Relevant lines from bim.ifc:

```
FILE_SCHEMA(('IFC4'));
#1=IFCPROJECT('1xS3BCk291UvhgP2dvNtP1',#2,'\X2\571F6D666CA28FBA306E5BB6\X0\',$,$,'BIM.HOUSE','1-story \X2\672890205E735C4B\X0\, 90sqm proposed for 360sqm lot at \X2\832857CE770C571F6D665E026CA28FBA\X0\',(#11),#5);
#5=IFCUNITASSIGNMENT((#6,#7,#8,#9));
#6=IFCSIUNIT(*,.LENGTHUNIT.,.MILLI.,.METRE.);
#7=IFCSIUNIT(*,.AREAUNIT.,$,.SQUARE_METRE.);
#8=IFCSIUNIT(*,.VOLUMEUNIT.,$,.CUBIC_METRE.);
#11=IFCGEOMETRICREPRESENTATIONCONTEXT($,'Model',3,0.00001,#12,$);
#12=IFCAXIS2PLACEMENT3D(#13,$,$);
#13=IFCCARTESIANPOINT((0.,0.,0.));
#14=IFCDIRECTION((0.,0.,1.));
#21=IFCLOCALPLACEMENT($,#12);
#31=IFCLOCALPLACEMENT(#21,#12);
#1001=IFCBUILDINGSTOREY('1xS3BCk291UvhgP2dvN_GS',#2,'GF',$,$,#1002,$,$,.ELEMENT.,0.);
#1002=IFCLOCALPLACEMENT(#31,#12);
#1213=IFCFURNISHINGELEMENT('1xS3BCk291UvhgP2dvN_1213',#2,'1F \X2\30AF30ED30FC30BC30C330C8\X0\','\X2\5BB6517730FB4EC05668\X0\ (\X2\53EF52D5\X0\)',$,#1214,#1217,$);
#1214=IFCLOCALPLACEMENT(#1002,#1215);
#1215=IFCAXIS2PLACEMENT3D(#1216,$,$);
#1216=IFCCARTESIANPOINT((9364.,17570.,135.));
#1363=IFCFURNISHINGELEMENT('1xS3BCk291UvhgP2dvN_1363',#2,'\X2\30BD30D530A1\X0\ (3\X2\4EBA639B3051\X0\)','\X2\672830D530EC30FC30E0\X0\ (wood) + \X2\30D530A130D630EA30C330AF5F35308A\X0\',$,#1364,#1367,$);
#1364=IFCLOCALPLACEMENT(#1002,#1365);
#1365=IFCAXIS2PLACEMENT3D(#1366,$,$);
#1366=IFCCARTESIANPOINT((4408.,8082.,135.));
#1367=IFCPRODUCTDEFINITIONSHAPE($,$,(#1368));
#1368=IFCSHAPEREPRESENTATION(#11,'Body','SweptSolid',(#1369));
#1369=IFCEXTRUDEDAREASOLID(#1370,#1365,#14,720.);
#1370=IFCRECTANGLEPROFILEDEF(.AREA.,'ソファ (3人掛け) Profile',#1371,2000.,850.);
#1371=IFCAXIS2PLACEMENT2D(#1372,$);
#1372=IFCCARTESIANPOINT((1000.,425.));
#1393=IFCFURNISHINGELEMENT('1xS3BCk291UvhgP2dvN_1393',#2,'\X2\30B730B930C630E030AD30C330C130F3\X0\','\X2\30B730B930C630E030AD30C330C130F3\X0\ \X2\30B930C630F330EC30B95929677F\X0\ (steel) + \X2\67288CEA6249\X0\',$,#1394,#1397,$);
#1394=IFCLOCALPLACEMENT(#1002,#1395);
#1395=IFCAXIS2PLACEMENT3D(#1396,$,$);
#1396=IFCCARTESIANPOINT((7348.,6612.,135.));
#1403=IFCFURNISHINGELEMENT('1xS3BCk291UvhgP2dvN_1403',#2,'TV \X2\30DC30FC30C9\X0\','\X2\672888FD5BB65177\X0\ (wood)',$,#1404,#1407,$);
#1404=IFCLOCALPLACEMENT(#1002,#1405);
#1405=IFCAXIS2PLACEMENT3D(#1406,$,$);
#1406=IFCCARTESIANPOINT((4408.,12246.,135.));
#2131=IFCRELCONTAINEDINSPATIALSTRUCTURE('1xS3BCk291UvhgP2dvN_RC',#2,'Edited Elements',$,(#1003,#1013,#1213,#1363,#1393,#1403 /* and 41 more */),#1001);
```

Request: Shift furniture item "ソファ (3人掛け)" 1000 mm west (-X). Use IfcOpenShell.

```python
import ifcopenshell
import ifcopenshell.api.geometry
import ifcopenshell.util.placement
import ifcopenshell.util.unit

model = ifcopenshell.open("bim.ifc")
unit_scale = ifcopenshell.util.unit.calculate_unit_scale(model)

item = model.by_guid("1xS3BCk291UvhgP2dvN_1363")
matrix = ifcopenshell.util.placement.get_local_placement(item.ObjectPlacement)
matrix[0, 3] -= 1 / unit_scale
ifcopenshell.api.geometry.edit_object_placement(model, product=item, matrix=matrix, is_si=False)

print(ifcopenshell.util.placement.get_local_placement(item.ObjectPlacement).round(3) + 0.0)

model.write("bim_edited.ifc")
```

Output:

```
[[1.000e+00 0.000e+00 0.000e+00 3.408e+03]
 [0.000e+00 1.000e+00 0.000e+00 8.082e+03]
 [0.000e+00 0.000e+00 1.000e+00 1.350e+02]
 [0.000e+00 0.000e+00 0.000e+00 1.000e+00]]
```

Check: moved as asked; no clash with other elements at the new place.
